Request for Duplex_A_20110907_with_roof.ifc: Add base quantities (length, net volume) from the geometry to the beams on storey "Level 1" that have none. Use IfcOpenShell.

First a look at what the model holds.

```python
import ifcopenshell
import ifcopenshell.util.element
import ifcopenshell.util.unit

model = ifcopenshell.open("Duplex_A_20110907_with_roof.ifc")
print(model.schema)
for unit_type in ("LENGTHUNIT", "AREAUNIT", "VOLUMEUNIT"):
    print(unit_type, ifcopenshell.util.unit.calculate_unit_scale(model, unit_type))
storey = next(s for s in model.by_type("IfcBuildingStorey") if s.Name == "Level 1")
beams = [e for e in ifcopenshell.util.element.get_decomposition(storey) if e.is_a("IfcBeam")]
for e in sorted(beams, key=lambda e: e.id()):
    print(e.id(), e.is_a(), e.Name, list(ifcopenshell.util.element.get_psets(e, qtos_only=True)), sep=" | ")
```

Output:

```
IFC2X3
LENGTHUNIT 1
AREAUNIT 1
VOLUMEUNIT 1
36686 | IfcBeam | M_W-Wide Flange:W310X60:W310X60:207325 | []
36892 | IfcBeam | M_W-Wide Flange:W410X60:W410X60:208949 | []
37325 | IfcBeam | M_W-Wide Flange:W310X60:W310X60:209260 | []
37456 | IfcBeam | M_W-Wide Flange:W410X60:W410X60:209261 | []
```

```python
import ifcopenshell
import ifcopenshell.api.pset
import ifcopenshell.geom
import ifcopenshell.util.element
import ifcopenshell.util.shape
import ifcopenshell.util.unit

model = ifcopenshell.open("Duplex_A_20110907_with_roof.ifc")
unit_scale = ifcopenshell.util.unit.calculate_unit_scale(model)
volume_scale = ifcopenshell.util.unit.calculate_unit_scale(model, "VOLUMEUNIT")
settings = ifcopenshell.geom.settings()

storey = next(s for s in model.by_type("IfcBuildingStorey") if s.Name == "Level 1")
beams = [e for e in ifcopenshell.util.element.get_decomposition(storey) if e.is_a("IfcBeam")]

for e in sorted(beams, key=lambda e: e.id()):
    if ifcopenshell.util.element.get_psets(e, qtos_only=True, should_inherit=False):
        continue
    # Geometry comes back in metres, in the element's own axes.
    shape = ifcopenshell.geom.create_shape(settings, e)
    values = {
        "Length": ifcopenshell.util.shape.get_max_xyz(shape.geometry) / unit_scale,
        "NetVolume": ifcopenshell.util.shape.get_volume(shape.geometry) / volume_scale,
    }
    qto = ifcopenshell.api.pset.add_qto(model, product=e, name="BaseQuantities")
    ifcopenshell.api.pset.edit_qto(model, qto=qto, properties=values)
    print(e.id(), {k: round(v, 3) for k, v in values.items()})

model.write("Duplex_A_20110907_with_roof_updated.ifc")
```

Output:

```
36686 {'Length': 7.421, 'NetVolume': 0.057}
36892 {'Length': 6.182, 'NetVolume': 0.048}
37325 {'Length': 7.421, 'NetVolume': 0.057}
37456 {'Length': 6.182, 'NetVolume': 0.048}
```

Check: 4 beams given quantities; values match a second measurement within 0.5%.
